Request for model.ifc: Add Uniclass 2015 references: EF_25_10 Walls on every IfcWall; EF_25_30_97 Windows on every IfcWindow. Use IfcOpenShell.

First a look at what the model holds.

```python
import ifcopenshell

model = ifcopenshell.open("model.ifc")
print(model.schema)
print("classifications:", [c.Name for c in model.by_type("IfcClassification")])
for ifc_class in ("IfcDoor", "IfcRoof", "IfcStair", "IfcWall", "IfcWindow"):
    print(ifc_class, len(model.by_type(ifc_class)))
```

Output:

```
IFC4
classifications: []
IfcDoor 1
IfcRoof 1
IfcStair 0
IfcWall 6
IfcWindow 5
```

```python
import ifcopenshell
import ifcopenshell.api.classification

model = ifcopenshell.open("model.ifc")

system = ifcopenshell.api.classification.add_classification(model, classification="Uniclass 2015")

codes = {
    "IfcWall": ("EF_25_10", "Walls"),
    "IfcWindow": ("EF_25_30_97", "Windows"),
}
for ifc_class, (code, name) in codes.items():
    products = model.by_type(ifc_class)
    ifcopenshell.api.classification.add_reference(
        model, products=products, classification=system, identification=code, name=name
    )
    print(code, len(products))

model.write("model_v2.ifc")
```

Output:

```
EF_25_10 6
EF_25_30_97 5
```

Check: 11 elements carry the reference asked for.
